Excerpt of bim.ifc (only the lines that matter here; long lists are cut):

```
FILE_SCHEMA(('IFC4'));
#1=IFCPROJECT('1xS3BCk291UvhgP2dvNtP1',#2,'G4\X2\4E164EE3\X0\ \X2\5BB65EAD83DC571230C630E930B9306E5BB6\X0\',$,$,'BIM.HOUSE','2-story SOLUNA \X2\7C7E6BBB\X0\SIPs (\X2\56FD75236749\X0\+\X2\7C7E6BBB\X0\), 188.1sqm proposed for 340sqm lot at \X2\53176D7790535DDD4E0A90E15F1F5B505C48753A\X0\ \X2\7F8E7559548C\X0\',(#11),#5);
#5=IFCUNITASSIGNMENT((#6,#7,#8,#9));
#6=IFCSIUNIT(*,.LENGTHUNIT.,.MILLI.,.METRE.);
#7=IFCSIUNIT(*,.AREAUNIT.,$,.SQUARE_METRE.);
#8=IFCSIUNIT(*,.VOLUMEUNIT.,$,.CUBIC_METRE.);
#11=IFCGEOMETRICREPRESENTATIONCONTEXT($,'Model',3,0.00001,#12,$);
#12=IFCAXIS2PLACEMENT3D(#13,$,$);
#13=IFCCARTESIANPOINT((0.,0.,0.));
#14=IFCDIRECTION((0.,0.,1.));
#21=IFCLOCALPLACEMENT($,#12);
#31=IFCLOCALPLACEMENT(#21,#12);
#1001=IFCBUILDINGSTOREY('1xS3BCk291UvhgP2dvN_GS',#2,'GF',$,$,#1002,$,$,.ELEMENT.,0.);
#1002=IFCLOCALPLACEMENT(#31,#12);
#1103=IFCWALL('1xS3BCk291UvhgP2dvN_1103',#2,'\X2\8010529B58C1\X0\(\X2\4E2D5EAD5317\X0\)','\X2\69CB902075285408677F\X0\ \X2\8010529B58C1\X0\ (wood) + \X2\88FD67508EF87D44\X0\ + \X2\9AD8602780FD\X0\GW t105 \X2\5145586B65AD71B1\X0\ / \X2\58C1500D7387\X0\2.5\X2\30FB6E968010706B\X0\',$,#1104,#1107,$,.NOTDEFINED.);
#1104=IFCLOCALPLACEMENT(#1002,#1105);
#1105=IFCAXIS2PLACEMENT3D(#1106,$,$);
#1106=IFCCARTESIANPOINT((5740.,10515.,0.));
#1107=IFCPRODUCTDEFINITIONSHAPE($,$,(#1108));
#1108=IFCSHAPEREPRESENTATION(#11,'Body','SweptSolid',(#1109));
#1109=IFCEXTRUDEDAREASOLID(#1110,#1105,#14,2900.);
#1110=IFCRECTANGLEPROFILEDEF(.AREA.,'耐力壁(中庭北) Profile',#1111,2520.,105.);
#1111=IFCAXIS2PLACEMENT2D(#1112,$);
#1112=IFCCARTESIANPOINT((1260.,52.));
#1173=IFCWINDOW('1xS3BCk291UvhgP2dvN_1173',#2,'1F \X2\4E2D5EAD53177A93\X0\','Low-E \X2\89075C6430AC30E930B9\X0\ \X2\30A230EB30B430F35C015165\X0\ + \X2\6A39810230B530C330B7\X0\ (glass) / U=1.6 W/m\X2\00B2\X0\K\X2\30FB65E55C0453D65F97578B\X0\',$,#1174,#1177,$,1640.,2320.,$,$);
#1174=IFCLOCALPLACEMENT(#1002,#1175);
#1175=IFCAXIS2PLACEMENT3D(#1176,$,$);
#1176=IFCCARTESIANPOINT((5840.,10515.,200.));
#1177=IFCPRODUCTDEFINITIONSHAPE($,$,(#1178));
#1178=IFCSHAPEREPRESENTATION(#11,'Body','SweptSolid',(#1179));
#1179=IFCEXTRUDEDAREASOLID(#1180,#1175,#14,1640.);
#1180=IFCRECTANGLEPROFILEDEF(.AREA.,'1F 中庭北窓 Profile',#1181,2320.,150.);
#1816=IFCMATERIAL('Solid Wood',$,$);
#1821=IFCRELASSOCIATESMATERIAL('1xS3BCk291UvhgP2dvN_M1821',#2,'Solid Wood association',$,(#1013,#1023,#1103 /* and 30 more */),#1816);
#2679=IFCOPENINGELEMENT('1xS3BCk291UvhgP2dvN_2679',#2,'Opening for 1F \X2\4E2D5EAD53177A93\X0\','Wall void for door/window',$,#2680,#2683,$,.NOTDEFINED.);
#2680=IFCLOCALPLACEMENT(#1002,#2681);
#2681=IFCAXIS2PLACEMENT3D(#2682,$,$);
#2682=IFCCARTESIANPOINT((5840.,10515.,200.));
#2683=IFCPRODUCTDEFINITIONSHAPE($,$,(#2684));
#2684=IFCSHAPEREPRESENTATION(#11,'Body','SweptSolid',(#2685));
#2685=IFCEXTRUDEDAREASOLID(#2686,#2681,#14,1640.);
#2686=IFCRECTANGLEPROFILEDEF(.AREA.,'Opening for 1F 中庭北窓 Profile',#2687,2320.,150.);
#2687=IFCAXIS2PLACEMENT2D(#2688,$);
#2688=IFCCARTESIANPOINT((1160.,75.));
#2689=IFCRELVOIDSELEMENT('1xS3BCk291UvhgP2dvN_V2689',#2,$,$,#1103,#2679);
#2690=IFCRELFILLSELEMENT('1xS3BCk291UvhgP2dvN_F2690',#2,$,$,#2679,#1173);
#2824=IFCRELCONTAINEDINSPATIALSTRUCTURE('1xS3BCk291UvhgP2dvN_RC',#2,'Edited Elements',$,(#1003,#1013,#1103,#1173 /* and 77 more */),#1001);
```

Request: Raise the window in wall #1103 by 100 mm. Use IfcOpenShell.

```python
import numpy as np
import ifcopenshell
import ifcopenshell.api.geometry
import ifcopenshell.util.placement
import ifcopenshell.util.unit

model = ifcopenshell.open("bim.ifc")
unit_scale = ifcopenshell.util.unit.calculate_unit_scale(model)

window = model.by_guid("1xS3BCk291UvhgP2dvN_1173")
opening = window.FillsVoids[0].RelatingOpeningElement
dz = 0.1 / unit_scale

shift = np.array([0.0, 0.0, dz])
# The window is not placed relative to its opening, so move both.
for product in (opening, window):
    matrix = ifcopenshell.util.placement.get_local_placement(product.ObjectPlacement)
    matrix[:3, 3] += shift
    ifcopenshell.api.geometry.edit_object_placement(model, product=product, matrix=matrix, is_si=False)

print(f"moved by {dz * unit_scale:+.3f} m")

model.write("bim_v2.ifc")
```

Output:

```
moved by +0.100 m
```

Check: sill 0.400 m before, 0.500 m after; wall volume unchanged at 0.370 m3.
